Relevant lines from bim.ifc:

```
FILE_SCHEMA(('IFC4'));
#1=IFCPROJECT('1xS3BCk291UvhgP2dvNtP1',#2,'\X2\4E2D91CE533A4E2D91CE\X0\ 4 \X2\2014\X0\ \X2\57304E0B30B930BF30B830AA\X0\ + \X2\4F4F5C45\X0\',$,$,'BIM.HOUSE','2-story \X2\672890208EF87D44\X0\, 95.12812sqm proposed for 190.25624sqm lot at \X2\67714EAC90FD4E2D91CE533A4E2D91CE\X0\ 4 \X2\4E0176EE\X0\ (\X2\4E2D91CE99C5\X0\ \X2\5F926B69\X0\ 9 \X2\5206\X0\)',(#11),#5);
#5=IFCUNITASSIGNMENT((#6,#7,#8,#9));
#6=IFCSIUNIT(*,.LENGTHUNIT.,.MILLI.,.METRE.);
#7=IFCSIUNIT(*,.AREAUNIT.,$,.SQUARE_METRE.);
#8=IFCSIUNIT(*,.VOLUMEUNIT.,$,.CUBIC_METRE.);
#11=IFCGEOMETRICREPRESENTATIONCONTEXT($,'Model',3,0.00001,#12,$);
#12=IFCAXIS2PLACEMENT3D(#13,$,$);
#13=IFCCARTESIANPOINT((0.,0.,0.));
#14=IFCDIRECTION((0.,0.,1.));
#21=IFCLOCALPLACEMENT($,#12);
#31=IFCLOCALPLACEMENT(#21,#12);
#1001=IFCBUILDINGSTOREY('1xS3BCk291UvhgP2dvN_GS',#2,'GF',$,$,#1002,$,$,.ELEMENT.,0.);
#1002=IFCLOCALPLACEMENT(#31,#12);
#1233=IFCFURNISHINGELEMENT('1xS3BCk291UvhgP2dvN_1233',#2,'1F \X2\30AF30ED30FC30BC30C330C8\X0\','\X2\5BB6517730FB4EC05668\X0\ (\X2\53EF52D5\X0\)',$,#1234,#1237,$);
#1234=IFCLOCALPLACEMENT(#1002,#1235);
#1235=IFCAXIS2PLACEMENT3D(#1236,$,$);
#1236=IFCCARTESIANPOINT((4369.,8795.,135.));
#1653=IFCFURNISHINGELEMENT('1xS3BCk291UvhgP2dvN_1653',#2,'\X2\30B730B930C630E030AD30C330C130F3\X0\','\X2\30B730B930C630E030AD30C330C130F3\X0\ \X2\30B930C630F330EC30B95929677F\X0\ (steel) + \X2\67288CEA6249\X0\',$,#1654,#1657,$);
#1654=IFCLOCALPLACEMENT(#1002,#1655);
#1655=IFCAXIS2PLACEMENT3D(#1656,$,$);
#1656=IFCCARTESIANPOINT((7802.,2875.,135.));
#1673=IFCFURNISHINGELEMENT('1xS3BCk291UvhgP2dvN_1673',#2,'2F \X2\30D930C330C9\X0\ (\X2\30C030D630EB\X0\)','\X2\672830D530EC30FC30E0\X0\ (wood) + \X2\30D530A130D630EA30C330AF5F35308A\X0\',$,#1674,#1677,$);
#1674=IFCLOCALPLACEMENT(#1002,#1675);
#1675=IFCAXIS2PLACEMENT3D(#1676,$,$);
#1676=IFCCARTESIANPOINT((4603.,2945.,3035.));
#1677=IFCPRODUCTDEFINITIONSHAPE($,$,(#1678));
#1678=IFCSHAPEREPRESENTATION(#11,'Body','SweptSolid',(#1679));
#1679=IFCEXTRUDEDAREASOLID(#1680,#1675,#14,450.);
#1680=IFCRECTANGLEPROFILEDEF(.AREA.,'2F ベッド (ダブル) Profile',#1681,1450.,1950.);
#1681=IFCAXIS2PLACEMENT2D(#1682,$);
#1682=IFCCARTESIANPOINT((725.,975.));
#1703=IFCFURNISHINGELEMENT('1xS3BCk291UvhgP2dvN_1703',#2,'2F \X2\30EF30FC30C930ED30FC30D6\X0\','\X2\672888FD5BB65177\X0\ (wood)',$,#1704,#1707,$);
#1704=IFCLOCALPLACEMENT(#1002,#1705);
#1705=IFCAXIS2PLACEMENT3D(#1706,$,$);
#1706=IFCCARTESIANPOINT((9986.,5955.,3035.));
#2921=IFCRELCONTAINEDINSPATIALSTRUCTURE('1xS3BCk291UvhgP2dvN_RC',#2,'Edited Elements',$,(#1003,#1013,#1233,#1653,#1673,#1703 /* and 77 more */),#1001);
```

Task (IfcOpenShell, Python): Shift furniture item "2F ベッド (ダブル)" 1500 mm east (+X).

```python
import ifcopenshell
import ifcopenshell.api.geometry
import ifcopenshell.util.placement
import ifcopenshell.util.unit

model = ifcopenshell.open("bim.ifc")
unit_scale = ifcopenshell.util.unit.calculate_unit_scale(model)

item = model.by_guid("1xS3BCk291UvhgP2dvN_1673")
matrix = ifcopenshell.util.placement.get_local_placement(item.ObjectPlacement)
matrix[0, 3] += 1.5 / unit_scale
ifcopenshell.api.geometry.edit_object_placement(model, product=item, matrix=matrix, is_si=False)

print(ifcopenshell.util.placement.get_local_placement(item.ObjectPlacement).round(3) + 0.0)

model.write("bim_edited.ifc")
```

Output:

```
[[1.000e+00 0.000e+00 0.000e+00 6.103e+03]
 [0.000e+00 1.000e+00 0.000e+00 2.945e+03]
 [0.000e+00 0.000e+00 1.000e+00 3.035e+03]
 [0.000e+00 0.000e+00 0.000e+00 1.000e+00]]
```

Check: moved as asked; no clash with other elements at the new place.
